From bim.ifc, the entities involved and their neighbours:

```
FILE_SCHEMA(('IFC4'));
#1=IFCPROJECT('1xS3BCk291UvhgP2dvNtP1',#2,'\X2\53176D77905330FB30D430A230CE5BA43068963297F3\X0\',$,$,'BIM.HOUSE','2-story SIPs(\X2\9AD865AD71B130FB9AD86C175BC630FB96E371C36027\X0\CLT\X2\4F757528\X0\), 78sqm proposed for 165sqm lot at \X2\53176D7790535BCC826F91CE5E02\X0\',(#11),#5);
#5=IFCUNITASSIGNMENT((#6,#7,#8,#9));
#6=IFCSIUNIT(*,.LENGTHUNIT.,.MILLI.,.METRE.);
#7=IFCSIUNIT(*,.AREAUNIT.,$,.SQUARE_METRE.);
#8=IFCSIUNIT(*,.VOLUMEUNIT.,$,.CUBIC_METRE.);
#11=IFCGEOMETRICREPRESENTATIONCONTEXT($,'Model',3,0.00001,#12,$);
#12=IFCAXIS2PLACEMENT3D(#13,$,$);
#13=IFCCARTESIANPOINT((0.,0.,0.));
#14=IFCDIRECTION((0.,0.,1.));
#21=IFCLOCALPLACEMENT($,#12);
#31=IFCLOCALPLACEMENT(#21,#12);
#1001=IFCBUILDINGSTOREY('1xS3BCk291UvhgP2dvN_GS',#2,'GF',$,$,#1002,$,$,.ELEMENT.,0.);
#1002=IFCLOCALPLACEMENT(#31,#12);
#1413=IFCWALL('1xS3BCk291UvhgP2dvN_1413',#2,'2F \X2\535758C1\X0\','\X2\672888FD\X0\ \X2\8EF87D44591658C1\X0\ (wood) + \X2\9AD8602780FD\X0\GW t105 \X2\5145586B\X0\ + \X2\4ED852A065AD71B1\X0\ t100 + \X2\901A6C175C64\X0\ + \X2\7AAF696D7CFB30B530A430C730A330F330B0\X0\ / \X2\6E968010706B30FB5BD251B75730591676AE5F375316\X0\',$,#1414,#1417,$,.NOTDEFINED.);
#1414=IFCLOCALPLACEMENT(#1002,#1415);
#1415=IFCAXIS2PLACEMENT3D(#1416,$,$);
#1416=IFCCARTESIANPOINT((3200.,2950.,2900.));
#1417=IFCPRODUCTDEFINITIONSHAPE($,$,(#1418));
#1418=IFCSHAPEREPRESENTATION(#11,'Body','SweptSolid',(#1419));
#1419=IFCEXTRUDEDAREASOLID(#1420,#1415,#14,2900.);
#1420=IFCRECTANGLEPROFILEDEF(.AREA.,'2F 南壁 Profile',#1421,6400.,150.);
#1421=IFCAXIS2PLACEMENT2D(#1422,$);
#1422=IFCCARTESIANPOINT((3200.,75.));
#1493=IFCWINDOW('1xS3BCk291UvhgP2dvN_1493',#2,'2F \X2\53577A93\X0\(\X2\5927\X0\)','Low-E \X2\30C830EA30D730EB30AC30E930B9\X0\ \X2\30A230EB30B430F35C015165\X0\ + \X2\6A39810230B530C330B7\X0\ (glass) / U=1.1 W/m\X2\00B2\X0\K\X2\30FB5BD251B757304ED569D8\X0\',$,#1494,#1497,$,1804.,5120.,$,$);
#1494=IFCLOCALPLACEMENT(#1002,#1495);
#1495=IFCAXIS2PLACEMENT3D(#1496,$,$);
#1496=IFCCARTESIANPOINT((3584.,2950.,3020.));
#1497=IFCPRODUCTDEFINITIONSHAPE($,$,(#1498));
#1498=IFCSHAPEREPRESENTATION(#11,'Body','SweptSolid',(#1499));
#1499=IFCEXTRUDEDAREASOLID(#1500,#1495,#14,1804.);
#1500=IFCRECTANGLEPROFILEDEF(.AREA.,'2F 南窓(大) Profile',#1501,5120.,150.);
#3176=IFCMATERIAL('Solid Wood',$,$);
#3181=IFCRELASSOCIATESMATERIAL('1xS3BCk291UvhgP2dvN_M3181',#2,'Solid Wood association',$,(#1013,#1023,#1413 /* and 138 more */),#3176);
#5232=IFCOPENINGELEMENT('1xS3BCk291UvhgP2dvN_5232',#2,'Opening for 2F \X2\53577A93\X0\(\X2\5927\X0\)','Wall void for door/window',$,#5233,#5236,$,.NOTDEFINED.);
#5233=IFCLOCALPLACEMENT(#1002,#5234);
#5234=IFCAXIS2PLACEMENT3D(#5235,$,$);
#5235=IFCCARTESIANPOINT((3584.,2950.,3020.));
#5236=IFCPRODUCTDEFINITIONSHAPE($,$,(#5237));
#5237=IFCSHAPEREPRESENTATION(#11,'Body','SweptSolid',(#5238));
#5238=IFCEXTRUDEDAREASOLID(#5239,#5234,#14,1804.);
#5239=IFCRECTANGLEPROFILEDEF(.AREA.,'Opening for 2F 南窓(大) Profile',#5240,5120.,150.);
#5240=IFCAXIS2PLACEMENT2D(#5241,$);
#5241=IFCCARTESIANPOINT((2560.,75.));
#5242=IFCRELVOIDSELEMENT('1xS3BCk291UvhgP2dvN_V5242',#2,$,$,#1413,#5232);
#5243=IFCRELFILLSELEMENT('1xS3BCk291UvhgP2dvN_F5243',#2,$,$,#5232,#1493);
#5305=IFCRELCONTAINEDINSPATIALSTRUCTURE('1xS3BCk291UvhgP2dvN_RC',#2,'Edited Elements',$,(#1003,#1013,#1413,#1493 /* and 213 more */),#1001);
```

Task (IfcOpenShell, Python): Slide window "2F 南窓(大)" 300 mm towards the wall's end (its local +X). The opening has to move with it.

```python
import ifcopenshell
import ifcopenshell.api.geometry
import ifcopenshell.util.placement
import ifcopenshell.util.unit

model = ifcopenshell.open("bim.ifc")
unit_scale = ifcopenshell.util.unit.calculate_unit_scale(model)

window = model.by_guid("1xS3BCk291UvhgP2dvN_1493")
opening = window.FillsVoids[0].RelatingOpeningElement
wall = opening.VoidsElements[0].RelatingBuildingElement

wall_matrix = ifcopenshell.util.placement.get_local_placement(wall.ObjectPlacement)
shift = wall_matrix[:3, 0] * 0.3 / unit_scale
before = ifcopenshell.util.placement.get_local_placement(window.ObjectPlacement)[:3, 3].copy()

# The window is not placed relative to its opening, so move both.
for product in (opening, window):
    matrix = ifcopenshell.util.placement.get_local_placement(product.ObjectPlacement)
    matrix[:3, 3] += shift
    ifcopenshell.api.geometry.edit_object_placement(model, product=product, matrix=matrix, is_si=False)

after = ifcopenshell.util.placement.get_local_placement(window.ObjectPlacement)[:3, 3]
print("window moved by", (after - before).round(3) + 0.0)

model.write("bim-out.ifc")
```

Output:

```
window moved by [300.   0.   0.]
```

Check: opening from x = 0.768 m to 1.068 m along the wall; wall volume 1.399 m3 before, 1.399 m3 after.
